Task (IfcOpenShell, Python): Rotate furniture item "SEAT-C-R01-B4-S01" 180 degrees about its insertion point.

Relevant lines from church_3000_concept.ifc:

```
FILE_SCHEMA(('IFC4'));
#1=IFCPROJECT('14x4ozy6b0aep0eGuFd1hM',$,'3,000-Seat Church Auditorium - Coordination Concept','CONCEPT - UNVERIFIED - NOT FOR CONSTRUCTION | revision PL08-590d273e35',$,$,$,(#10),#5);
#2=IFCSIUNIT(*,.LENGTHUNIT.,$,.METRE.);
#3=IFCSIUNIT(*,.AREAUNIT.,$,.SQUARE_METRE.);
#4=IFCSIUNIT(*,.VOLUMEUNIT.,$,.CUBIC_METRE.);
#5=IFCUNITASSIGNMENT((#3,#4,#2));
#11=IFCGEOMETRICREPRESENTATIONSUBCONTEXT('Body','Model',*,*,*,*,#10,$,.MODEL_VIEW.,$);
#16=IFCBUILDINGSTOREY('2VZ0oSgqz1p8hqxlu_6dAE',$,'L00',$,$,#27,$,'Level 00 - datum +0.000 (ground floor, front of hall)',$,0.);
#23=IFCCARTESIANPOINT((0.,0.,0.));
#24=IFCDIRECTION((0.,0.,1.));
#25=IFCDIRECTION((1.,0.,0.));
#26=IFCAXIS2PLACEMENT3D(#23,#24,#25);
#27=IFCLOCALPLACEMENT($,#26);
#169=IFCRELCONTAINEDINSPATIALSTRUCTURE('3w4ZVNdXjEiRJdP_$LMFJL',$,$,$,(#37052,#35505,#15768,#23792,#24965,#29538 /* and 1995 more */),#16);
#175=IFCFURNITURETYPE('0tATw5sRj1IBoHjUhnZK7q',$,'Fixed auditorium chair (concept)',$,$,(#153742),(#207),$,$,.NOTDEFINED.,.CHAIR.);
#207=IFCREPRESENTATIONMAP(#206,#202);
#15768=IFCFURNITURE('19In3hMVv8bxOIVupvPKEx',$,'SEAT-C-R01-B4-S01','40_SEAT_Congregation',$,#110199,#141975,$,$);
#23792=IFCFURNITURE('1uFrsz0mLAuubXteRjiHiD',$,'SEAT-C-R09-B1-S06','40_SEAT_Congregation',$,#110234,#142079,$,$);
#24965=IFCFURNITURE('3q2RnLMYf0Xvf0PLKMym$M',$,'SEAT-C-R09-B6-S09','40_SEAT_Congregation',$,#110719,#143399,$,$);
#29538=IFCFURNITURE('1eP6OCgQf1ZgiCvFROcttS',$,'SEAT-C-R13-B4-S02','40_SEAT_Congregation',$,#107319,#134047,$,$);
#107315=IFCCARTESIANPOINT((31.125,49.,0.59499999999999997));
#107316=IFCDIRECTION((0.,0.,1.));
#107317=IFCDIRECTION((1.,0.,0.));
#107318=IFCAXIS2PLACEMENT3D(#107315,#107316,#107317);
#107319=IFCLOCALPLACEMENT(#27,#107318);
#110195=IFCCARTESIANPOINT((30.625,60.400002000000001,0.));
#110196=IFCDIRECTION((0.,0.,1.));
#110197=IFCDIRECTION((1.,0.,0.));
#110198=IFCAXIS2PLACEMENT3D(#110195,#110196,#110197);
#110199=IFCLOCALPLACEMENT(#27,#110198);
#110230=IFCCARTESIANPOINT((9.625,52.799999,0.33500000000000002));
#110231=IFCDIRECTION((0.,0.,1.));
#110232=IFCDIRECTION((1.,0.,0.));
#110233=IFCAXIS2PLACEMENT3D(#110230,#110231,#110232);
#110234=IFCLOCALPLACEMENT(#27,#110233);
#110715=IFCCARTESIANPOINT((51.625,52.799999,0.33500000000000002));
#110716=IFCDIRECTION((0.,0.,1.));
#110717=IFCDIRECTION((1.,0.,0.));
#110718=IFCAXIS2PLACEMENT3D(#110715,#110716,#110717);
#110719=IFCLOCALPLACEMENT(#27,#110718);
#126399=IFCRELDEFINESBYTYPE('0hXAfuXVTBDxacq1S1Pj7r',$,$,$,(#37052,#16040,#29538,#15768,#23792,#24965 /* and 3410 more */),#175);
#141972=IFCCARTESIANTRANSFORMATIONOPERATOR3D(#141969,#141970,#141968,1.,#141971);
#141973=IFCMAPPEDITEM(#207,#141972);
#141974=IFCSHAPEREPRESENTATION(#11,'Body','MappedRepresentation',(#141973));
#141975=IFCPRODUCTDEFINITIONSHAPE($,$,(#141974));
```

```python
import ifcopenshell
import ifcopenshell.api.geometry
import ifcopenshell.util.placement

model = ifcopenshell.open("church_3000_concept.ifc")

item = model.by_id(15768)
matrix = ifcopenshell.util.placement.get_local_placement(item.ObjectPlacement)
matrix = matrix @ ifcopenshell.util.placement.rotation(180, "Z")
ifcopenshell.api.geometry.edit_object_placement(model, product=item, matrix=matrix, is_si=False)

print(ifcopenshell.util.placement.get_local_placement(item.ObjectPlacement).round(3) + 0.0)

model.write("church_3000_concept_edited.ifc")
```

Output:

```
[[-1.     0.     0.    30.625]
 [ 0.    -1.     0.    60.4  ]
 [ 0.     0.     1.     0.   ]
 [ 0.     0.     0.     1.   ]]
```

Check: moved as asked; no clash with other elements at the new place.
